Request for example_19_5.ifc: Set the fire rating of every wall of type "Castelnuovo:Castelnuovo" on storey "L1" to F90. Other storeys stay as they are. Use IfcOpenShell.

First a look at what the model holds.

```python
import ifcopenshell
import ifcopenshell.util.element

model = ifcopenshell.open("example_19_5.ifc")
print(model.schema)
storey = next(s for s in model.by_type("IfcBuildingStorey") if s.Name == "L1")
walls = [e for e in ifcopenshell.util.element.get_decomposition(storey) if e.is_a("IfcWall")]
seen = {}
for e in walls:
    element_type = ifcopenshell.util.element.get_type(e)
    key = (element_type.Name if element_type != e and element_type else None, ifcopenshell.util.element.get_pset(e, "Pset_WallCommon", "FireRating"))
    seen[key] = seen.get(key, 0) + 1
for (name, value), count in sorted(seen.items(), key=str):
    print(count, "x", name, "|", value)
```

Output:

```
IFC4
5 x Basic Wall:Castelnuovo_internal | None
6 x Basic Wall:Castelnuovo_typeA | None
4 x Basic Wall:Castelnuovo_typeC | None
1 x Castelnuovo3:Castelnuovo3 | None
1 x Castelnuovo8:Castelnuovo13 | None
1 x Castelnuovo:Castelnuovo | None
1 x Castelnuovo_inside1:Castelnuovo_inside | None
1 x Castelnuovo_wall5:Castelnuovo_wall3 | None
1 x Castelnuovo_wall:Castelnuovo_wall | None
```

```python
import ifcopenshell
import ifcopenshell.api.pset
import ifcopenshell.util.element

model = ifcopenshell.open("example_19_5.ifc")

storey = next(s for s in model.by_type("IfcBuildingStorey") if s.Name == "L1")
walls = [e for e in ifcopenshell.util.element.get_decomposition(storey) if e.is_a("IfcWall")]

count = 0
for e in walls:
    element_type = ifcopenshell.util.element.get_type(e)
    if element_type in (None, e) or element_type.Name != "Castelnuovo:Castelnuovo":
        continue
    # add_pset returns the element's existing set when there is one.
    pset = ifcopenshell.api.pset.add_pset(model, product=e, name="Pset_WallCommon")
    ifcopenshell.api.pset.edit_pset(model, pset=pset, properties={"FireRating": "F90"})
    count += 1

print(count, "walls updated")

model.write("example_19_5_edited.ifc")
```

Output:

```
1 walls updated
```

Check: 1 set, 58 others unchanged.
